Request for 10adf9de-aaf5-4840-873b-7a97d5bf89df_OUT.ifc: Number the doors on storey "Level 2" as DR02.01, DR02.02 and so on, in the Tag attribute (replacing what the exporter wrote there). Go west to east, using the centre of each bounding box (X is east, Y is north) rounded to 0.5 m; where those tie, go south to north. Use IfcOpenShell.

First a look at what the model holds.

```python
import ifcopenshell
import ifcopenshell.util.element
import ifcopenshell.util.placement

model = ifcopenshell.open("10adf9de-aaf5-4840-873b-7a97d5bf89df_OUT.ifc")
print(model.schema)
storey = next(s for s in model.by_type("IfcBuildingStorey") if s.Name == "Level 2")
doors = [e for e in ifcopenshell.util.element.get_decomposition(storey) if e.is_a("IfcDoor")]
for e in sorted(doors, key=lambda e: e.id()):
    origin = ifcopenshell.util.placement.get_local_placement(e.ObjectPlacement)[:3, 3]
    print(e.id(), e.Tag, e.Name, origin.round(2) + 0.0, sep=" | ")
```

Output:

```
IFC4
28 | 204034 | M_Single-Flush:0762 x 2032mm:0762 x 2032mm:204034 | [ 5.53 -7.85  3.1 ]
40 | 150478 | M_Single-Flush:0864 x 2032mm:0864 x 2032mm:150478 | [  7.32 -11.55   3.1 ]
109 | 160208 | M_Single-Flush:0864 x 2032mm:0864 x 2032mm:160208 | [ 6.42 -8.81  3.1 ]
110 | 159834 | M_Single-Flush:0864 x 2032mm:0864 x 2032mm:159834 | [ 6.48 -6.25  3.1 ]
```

```python
import ifcopenshell
import ifcopenshell.geom
import ifcopenshell.util.element
import ifcopenshell.util.shape

model = ifcopenshell.open("10adf9de-aaf5-4840-873b-7a97d5bf89df_OUT.ifc")
settings = ifcopenshell.geom.settings()
settings.set("use-world-coords", True)


def centre(element):
    shape = ifcopenshell.geom.create_shape(settings, element)
    return ifcopenshell.util.shape.get_bbox_centroid(shape.geometry)


storey = next(s for s in model.by_type("IfcBuildingStorey") if s.Name == "Level 2")
doors = [e for e in ifcopenshell.util.element.get_decomposition(storey) if e.is_a("IfcDoor")]

# Insertion points can sit at a corner or the storey origin, so sort by the geometry (in metres).
centres = {e: centre(e) for e in doors}
doors.sort(key=lambda e: (round(centres[e][0] / 0.5), centres[e][1]))

for i, e in enumerate(doors, start=1):
    number = f"DR02.{i:02d}"
    e.Tag = number
    print(e.id(), number)

model.write("10adf9de-aaf5-4840-873b-7a97d5bf89df_OUT_edited.ifc")
```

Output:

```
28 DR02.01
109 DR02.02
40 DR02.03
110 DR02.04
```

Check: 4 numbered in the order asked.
